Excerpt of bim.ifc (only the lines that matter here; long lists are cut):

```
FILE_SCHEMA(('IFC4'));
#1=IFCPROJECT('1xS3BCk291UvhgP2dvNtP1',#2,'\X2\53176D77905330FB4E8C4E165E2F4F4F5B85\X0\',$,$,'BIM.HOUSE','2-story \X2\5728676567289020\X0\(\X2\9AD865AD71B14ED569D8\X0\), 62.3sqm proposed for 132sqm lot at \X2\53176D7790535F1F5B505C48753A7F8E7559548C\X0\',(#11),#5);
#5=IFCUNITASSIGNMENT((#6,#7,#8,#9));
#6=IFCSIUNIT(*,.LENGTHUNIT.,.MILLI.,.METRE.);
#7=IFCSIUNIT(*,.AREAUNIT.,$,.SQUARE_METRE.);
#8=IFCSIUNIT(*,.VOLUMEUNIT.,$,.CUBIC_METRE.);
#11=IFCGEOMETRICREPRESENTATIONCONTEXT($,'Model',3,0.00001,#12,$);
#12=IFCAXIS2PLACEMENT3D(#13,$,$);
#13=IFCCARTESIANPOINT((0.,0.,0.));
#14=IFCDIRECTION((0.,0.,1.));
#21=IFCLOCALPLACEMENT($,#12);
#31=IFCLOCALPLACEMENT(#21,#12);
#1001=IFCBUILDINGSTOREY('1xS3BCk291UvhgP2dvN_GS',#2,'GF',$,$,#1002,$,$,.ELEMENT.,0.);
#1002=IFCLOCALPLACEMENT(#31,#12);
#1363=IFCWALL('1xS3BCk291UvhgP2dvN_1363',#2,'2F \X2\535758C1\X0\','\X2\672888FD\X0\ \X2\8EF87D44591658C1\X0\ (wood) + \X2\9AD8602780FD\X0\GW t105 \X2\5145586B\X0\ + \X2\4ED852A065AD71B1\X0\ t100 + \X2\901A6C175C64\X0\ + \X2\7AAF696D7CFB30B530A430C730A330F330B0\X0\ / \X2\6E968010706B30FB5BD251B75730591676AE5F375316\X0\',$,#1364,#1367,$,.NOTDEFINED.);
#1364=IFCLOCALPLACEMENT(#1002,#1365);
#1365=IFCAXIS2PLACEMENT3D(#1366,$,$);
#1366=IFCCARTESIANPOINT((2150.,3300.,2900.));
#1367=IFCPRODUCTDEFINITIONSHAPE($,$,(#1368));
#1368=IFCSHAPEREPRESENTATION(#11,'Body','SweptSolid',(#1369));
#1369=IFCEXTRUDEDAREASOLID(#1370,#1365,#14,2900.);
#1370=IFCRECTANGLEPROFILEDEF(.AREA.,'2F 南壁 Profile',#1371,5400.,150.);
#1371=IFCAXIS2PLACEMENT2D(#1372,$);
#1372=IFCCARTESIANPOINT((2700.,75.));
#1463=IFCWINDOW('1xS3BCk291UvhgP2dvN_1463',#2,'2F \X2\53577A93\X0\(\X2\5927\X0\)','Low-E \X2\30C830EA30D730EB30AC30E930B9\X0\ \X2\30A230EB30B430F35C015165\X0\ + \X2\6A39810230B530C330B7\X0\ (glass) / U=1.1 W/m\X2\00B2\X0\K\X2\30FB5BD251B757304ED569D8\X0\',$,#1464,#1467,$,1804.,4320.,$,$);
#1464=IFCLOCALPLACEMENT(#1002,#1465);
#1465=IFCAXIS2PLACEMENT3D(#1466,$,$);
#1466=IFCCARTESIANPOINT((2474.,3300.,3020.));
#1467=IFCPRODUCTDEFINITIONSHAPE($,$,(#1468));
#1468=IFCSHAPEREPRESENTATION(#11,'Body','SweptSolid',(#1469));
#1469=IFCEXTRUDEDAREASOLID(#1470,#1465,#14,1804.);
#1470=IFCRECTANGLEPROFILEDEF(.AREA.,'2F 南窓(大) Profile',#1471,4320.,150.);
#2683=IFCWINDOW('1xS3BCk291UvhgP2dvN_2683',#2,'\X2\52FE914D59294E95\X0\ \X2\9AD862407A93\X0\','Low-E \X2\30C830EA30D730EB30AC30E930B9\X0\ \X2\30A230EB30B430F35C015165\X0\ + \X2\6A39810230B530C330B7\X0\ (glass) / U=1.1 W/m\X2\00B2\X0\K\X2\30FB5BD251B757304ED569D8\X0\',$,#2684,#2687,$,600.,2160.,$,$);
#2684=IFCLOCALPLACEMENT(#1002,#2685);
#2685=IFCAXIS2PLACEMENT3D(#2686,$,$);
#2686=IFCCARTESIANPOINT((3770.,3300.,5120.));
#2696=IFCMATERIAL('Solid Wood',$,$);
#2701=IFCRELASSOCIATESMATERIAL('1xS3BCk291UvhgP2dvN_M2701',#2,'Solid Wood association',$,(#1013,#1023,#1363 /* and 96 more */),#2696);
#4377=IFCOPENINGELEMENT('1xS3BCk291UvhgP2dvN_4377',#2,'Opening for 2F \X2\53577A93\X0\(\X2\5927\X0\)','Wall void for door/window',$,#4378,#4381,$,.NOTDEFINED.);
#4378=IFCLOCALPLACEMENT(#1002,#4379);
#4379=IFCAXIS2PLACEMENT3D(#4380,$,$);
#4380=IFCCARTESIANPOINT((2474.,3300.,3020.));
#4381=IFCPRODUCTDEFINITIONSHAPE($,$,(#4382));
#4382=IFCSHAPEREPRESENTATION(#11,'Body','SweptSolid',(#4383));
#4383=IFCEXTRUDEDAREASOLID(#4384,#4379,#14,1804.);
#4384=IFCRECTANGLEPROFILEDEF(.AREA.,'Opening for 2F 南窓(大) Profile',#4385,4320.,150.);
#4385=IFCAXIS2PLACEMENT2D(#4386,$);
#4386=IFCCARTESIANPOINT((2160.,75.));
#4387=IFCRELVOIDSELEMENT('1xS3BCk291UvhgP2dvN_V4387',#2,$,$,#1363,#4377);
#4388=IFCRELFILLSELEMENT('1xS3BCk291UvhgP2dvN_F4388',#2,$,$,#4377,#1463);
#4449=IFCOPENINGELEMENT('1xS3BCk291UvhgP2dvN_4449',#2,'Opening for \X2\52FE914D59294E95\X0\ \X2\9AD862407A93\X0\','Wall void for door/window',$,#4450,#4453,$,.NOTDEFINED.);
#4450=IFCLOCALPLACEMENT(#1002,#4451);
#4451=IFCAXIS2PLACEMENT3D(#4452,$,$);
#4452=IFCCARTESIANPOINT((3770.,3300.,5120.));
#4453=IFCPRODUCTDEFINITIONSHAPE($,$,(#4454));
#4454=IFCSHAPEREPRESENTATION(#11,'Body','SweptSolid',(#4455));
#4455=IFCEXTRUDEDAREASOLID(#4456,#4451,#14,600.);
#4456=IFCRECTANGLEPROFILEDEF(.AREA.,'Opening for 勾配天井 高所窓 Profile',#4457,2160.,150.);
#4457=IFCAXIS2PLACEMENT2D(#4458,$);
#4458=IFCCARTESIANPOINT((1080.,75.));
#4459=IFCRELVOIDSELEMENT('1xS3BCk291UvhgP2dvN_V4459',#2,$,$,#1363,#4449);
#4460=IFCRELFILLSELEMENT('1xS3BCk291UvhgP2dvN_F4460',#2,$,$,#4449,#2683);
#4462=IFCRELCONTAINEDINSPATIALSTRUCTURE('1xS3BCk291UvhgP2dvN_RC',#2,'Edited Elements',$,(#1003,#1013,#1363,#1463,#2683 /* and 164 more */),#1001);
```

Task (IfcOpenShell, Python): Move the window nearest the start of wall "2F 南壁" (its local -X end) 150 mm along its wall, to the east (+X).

```python
import ifcopenshell
import ifcopenshell.api.geometry
import ifcopenshell.util.placement

model = ifcopenshell.open("bim.ifc")

window = model.by_id(1463)
opening = window.FillsVoids[0].RelatingOpeningElement
wall = opening.VoidsElements[0].RelatingBuildingElement

wall_matrix = ifcopenshell.util.placement.get_local_placement(wall.ObjectPlacement)
shift = wall_matrix[:3, 0] * 150.0
before = ifcopenshell.util.placement.get_local_placement(window.ObjectPlacement)[:3, 3].copy()

# The window is not placed relative to its opening, so move both.
for product in (opening, window):
    matrix = ifcopenshell.util.placement.get_local_placement(product.ObjectPlacement)
    matrix[:3, 3] += shift
    ifcopenshell.api.geometry.edit_object_placement(model, product=product, matrix=matrix, is_si=False)

after = ifcopenshell.util.placement.get_local_placement(window.ObjectPlacement)[:3, 3]
print("window moved by", (after - before).round(3) + 0.0)

model.write("bim_v2.ifc")
```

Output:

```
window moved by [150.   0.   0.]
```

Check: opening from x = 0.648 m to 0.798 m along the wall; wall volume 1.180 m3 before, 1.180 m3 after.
